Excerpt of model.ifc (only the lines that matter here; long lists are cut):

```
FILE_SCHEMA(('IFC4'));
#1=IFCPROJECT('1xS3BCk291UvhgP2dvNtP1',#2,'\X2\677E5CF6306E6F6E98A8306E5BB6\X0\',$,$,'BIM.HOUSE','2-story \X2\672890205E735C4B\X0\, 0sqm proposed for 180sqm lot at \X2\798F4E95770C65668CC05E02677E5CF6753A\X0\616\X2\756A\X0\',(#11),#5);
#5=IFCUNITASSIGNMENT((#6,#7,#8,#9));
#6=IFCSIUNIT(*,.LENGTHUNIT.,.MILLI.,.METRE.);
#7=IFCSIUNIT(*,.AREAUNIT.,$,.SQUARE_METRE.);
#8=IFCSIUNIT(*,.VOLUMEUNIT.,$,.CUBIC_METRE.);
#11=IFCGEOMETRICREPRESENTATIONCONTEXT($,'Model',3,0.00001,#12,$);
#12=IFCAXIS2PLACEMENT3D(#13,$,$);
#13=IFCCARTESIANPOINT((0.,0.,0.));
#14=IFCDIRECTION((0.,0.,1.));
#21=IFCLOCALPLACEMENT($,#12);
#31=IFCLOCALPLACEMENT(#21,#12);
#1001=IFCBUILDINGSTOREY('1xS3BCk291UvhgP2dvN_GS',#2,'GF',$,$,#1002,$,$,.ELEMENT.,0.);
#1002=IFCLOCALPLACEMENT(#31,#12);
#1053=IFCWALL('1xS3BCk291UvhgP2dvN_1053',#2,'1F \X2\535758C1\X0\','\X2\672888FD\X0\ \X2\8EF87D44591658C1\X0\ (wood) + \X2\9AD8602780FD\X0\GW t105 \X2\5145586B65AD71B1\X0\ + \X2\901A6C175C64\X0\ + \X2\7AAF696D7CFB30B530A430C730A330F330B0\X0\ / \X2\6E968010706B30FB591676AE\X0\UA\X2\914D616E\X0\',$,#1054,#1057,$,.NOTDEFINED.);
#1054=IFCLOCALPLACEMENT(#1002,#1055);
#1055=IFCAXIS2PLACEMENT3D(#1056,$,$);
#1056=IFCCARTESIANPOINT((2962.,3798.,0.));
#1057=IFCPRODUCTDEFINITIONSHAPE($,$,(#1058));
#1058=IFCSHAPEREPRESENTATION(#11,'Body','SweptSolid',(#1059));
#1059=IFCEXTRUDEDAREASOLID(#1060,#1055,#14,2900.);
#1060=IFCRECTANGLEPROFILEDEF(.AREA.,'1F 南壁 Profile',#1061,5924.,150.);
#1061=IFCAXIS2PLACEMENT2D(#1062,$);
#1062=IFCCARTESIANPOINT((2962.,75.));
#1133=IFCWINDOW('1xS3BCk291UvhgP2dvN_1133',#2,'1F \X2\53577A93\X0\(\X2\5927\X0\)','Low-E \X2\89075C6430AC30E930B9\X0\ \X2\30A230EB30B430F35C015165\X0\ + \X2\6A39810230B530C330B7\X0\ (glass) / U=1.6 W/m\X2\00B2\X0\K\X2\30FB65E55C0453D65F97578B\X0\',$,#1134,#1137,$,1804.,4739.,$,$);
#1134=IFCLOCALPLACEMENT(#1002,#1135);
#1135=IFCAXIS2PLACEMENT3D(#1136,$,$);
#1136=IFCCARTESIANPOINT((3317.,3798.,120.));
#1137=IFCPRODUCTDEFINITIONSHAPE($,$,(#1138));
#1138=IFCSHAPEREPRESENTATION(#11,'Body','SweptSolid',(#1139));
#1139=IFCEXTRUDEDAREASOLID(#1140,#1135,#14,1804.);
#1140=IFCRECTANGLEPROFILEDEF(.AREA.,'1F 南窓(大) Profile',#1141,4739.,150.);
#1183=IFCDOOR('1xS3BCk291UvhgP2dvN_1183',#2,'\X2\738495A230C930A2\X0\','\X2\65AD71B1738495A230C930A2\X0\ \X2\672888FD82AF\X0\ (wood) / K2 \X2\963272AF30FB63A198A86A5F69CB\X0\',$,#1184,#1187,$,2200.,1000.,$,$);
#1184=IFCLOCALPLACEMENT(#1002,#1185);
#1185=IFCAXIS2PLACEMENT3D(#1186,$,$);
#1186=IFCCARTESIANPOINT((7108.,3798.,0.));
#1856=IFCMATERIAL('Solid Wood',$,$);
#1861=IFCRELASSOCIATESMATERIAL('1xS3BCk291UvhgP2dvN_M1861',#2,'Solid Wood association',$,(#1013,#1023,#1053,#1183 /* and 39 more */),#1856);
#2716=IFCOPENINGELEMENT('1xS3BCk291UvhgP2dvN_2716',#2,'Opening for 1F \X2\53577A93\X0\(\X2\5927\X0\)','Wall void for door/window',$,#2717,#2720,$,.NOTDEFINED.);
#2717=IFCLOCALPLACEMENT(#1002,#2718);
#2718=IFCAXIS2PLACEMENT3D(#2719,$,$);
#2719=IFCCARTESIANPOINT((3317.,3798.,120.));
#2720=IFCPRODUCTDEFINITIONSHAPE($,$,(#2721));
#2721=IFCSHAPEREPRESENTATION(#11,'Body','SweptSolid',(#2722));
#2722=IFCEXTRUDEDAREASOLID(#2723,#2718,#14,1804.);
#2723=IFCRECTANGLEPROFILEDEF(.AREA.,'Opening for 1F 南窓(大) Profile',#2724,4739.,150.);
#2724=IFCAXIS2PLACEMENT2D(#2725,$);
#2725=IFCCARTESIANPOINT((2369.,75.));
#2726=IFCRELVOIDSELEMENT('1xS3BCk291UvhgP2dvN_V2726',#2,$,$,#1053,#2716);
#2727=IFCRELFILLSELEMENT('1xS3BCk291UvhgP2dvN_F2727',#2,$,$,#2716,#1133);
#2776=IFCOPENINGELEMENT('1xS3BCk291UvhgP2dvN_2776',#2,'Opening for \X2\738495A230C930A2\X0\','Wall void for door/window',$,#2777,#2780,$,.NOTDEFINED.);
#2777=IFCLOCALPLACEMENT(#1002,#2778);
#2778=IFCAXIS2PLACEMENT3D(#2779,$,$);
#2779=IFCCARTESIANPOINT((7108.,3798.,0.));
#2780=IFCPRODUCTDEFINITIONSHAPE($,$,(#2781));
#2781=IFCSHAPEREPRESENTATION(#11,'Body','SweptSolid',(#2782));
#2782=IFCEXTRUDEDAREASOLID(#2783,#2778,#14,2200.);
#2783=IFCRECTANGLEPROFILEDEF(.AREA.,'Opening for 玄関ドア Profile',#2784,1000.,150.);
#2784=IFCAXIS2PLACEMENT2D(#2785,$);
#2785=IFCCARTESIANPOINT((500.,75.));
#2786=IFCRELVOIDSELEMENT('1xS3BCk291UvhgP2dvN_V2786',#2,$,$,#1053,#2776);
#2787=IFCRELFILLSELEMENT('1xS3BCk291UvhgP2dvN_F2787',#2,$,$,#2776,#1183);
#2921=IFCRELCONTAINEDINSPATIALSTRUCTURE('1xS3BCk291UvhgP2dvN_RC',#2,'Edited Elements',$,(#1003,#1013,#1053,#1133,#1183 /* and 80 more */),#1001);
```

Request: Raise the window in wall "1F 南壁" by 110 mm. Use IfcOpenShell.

```python
import numpy as np
import ifcopenshell
import ifcopenshell.api.geometry
import ifcopenshell.util.placement
import ifcopenshell.util.unit

model = ifcopenshell.open("model.ifc")
unit_scale = ifcopenshell.util.unit.calculate_unit_scale(model)

window = model.by_guid("1xS3BCk291UvhgP2dvN_1133")
opening = window.FillsVoids[0].RelatingOpeningElement
dz = 110.0

shift = np.array([0.0, 0.0, dz])
# The window is not placed relative to its opening, so move both.
for product in (opening, window):
    matrix = ifcopenshell.util.placement.get_local_placement(product.ObjectPlacement)
    matrix[:3, 3] += shift
    ifcopenshell.api.geometry.edit_object_placement(model, product=product, matrix=matrix, is_si=False)

print(f"moved by {dz * unit_scale:+.3f} m")

model.write("model_edited.ifc")
```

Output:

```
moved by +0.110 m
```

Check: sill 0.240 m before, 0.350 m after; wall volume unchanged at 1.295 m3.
